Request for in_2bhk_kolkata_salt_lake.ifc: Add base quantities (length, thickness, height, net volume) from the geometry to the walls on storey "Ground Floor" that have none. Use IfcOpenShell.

First a look at what the model holds.

```python
import ifcopenshell
import ifcopenshell.util.element
import ifcopenshell.util.unit

model = ifcopenshell.open("in_2bhk_kolkata_salt_lake.ifc")
print(model.schema)
for unit_type in ("LENGTHUNIT", "AREAUNIT", "VOLUMEUNIT"):
    print(unit_type, ifcopenshell.util.unit.calculate_unit_scale(model, unit_type))
storey = next(s for s in model.by_type("IfcBuildingStorey") if s.Name == "Ground Floor")
walls = [e for e in ifcopenshell.util.element.get_decomposition(storey) if e.is_a("IfcWall")]
for e in sorted(walls, key=lambda e: e.id()):
    print(e.id(), e.is_a(), e.Name, list(ifcopenshell.util.element.get_psets(e, qtos_only=True)), sep=" | ")
```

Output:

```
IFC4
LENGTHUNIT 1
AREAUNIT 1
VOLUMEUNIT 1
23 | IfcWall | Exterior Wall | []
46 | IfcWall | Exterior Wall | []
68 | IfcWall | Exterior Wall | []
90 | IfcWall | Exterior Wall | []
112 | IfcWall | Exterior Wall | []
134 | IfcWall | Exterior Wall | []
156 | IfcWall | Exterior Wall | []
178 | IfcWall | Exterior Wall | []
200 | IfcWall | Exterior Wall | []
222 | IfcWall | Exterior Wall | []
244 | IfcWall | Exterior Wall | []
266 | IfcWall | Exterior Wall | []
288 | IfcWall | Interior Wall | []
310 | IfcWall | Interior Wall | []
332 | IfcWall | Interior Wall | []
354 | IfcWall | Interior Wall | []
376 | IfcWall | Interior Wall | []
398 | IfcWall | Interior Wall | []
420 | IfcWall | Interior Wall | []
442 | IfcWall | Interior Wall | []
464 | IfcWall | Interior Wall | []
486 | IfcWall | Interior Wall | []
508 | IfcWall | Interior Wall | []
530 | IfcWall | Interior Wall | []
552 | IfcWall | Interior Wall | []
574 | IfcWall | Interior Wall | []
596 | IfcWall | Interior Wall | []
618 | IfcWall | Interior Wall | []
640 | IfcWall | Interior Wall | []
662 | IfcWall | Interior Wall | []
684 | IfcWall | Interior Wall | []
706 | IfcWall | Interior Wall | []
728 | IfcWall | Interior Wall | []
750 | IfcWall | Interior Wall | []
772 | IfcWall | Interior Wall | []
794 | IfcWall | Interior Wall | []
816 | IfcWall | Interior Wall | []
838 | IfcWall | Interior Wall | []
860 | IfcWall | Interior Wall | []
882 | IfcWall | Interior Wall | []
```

```python
import ifcopenshell
import ifcopenshell.api.pset
import ifcopenshell.geom
import ifcopenshell.util.element
import ifcopenshell.util.shape
import ifcopenshell.util.unit

model = ifcopenshell.open("in_2bhk_kolkata_salt_lake.ifc")
unit_scale = ifcopenshell.util.unit.calculate_unit_scale(model)
volume_scale = ifcopenshell.util.unit.calculate_unit_scale(model, "VOLUMEUNIT")
settings = ifcopenshell.geom.settings()

storey = next(s for s in model.by_type("IfcBuildingStorey") if s.Name == "Ground Floor")
walls = [e for e in ifcopenshell.util.element.get_decomposition(storey) if e.is_a("IfcWall")]

for e in sorted(walls, key=lambda e: e.id()):
    if ifcopenshell.util.element.get_psets(e, qtos_only=True, should_inherit=False):
        continue
    # Geometry comes back in metres, in the element's own axes.
    shape = ifcopenshell.geom.create_shape(settings, e)
    values = {
        "Length": ifcopenshell.util.shape.get_x(shape.geometry) / unit_scale,
        "Width": ifcopenshell.util.shape.get_y(shape.geometry) / unit_scale,
        "Height": ifcopenshell.util.shape.get_z(shape.geometry) / unit_scale,
        "NetVolume": ifcopenshell.util.shape.get_volume(shape.geometry) / volume_scale,
    }
    qto = ifcopenshell.api.pset.add_qto(model, product=e, name="Qto_WallBaseQuantities")
    ifcopenshell.api.pset.edit_qto(model, qto=qto, properties=values)
    print(e.id(), {k: round(v, 3) for k, v in values.items()})

model.write("in_2bhk_kolkata_salt_lake-out.ifc")
```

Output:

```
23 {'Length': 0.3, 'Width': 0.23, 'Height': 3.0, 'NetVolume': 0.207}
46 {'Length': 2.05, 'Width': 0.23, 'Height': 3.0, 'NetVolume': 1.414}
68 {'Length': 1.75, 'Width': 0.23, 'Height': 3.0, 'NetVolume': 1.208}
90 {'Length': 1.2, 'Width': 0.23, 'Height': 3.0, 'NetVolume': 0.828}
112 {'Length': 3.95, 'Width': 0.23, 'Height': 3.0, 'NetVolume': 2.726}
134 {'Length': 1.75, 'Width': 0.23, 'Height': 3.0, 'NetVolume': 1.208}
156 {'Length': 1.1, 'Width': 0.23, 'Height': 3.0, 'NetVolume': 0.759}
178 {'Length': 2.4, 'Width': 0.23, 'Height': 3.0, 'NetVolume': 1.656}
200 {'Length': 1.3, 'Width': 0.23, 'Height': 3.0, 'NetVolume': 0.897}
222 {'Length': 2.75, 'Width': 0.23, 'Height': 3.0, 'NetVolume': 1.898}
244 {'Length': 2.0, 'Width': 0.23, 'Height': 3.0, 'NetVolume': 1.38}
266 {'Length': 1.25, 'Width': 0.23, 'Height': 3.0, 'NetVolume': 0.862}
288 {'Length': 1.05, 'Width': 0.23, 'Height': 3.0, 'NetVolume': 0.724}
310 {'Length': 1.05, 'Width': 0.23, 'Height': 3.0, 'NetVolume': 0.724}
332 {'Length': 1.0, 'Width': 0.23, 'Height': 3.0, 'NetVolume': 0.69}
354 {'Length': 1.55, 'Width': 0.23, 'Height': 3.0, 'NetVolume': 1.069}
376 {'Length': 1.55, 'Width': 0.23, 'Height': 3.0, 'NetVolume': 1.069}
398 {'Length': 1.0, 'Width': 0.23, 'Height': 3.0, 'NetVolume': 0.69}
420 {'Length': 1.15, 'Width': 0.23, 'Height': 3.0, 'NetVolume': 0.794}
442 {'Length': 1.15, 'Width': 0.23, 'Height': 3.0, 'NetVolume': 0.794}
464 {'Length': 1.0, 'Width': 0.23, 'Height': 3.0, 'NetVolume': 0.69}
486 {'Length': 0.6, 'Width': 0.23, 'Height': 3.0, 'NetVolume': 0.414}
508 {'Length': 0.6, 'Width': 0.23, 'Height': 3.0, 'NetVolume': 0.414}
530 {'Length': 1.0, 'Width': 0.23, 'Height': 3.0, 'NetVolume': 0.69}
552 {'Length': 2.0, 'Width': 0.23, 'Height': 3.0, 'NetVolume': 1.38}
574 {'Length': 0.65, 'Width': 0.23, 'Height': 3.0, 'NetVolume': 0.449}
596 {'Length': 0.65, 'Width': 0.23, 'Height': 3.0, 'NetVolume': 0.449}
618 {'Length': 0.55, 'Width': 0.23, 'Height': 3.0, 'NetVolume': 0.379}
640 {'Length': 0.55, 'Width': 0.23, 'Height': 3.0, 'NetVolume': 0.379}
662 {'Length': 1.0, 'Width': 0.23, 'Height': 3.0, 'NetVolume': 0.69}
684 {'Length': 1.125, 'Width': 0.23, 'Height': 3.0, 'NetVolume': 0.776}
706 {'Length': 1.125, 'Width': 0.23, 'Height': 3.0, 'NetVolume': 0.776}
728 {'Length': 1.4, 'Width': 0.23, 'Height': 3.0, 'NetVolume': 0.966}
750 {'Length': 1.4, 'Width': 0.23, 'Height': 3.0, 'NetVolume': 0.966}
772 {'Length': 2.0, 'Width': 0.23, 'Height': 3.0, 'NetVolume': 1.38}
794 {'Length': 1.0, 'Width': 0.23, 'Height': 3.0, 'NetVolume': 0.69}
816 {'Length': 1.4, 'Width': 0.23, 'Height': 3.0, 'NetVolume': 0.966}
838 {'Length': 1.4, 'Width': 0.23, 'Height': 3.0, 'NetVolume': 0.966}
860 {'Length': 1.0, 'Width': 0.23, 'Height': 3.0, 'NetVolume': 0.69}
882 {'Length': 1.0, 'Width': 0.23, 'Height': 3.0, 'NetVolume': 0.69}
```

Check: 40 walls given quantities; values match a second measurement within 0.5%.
